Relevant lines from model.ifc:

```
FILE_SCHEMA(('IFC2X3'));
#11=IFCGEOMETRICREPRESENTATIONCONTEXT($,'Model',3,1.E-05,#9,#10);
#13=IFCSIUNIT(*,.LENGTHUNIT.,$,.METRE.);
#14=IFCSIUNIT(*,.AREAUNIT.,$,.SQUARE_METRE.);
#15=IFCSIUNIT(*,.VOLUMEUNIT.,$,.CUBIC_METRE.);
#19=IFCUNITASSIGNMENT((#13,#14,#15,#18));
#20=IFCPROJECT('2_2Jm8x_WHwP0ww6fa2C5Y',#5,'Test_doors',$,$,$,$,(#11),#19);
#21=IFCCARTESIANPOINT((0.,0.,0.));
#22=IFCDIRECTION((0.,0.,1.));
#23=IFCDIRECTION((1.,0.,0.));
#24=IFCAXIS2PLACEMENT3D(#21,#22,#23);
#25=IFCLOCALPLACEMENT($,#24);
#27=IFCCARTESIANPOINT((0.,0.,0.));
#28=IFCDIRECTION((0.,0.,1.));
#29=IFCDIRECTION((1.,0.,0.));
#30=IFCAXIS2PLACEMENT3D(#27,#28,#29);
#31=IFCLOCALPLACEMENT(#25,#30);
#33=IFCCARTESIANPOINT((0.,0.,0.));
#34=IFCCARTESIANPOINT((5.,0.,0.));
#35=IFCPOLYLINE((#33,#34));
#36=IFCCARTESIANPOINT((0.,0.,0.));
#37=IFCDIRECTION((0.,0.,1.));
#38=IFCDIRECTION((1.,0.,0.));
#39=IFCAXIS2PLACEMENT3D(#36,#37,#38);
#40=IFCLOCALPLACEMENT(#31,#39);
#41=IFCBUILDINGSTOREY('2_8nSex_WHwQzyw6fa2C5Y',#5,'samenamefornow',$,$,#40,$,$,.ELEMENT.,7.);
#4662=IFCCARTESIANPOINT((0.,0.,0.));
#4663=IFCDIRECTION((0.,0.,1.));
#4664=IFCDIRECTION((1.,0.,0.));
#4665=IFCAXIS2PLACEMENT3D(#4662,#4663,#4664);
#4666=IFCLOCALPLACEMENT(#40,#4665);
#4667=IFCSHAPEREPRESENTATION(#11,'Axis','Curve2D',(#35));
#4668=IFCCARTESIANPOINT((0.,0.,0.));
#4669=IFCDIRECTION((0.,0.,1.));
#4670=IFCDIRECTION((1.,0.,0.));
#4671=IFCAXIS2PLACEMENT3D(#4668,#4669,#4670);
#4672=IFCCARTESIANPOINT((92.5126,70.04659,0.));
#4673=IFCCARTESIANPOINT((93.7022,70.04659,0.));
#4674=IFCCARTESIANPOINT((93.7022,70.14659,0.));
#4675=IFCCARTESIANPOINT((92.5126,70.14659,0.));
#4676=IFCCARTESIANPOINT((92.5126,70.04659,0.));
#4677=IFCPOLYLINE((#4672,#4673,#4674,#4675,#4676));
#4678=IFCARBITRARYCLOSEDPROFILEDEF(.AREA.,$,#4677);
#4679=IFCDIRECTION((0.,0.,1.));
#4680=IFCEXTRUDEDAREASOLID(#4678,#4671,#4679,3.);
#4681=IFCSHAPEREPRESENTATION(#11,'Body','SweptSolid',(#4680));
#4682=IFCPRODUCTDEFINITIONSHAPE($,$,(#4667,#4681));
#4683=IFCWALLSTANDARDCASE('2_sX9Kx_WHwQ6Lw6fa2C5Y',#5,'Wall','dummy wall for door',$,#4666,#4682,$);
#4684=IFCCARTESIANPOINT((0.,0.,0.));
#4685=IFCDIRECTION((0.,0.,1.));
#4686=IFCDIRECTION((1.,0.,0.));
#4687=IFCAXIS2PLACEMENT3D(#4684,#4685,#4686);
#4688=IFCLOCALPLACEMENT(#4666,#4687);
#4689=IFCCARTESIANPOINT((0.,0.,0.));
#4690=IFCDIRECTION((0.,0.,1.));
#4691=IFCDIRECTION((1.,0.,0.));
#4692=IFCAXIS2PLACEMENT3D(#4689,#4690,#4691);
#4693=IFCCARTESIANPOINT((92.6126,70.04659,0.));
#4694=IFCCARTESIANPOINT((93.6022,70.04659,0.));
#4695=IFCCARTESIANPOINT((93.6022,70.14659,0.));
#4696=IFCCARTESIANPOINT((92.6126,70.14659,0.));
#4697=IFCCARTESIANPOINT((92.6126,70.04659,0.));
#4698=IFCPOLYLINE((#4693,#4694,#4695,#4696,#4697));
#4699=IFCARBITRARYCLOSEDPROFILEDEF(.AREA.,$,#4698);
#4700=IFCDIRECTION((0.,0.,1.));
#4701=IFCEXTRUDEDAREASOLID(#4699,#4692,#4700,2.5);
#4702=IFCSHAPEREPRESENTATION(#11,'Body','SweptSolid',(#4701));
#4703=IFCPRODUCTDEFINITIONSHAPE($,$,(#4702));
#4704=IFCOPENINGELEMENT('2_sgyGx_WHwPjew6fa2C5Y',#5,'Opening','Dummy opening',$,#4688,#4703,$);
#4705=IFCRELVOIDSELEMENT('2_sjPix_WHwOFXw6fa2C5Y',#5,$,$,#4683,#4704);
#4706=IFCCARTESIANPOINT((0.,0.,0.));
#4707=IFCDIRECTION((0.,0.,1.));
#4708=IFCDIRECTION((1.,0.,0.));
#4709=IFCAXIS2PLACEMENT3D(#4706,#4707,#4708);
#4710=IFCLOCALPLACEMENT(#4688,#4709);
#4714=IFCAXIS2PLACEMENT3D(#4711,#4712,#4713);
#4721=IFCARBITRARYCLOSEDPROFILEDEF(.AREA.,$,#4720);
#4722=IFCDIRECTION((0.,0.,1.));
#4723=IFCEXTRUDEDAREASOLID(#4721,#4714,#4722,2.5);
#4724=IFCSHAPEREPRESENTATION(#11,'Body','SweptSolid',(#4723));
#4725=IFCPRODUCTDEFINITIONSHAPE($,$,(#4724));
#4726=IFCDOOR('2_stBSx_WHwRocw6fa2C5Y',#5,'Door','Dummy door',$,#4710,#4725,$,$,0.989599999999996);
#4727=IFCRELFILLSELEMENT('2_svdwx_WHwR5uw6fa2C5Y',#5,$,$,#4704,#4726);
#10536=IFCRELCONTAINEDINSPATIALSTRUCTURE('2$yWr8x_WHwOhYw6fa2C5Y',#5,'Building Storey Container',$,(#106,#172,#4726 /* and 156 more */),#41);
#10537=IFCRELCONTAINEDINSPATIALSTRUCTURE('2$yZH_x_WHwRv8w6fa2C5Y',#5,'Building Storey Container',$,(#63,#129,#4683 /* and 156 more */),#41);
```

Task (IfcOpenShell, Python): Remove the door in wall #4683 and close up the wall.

```python
import ifcopenshell
import ifcopenshell.api.feature
import ifcopenshell.api.root
import ifcopenshell.geom
import ifcopenshell.util.shape

model = ifcopenshell.open("model.ifc")
settings = ifcopenshell.geom.settings()


def volume(element):
    """Net volume in cubic metres, openings subtracted."""
    shape = ifcopenshell.geom.create_shape(settings, element)
    return ifcopenshell.util.shape.get_volume(shape.geometry)


door = model.by_guid("2_stBSx_WHwRocw6fa2C5Y")
opening = door.FillsVoids[0].RelatingOpeningElement
wall = opening.VoidsElements[0].RelatingBuildingElement
before = volume(wall)

ifcopenshell.api.root.remove_product(model, product=door)
ifcopenshell.api.feature.remove_feature(model, feature=opening)

after = volume(wall)

print(f"wall volume {before:.3f} -> {after:.3f} m3")

model.write("model-out.ifc")
```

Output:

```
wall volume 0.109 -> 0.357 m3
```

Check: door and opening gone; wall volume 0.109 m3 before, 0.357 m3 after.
